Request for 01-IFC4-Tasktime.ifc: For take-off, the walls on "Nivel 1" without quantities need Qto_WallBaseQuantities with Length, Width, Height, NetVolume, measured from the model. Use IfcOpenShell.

First a look at what the model holds.

```python
import ifcopenshell
import ifcopenshell.util.element
import ifcopenshell.util.unit

model = ifcopenshell.open("01-IFC4-Tasktime.ifc")
print(model.schema)
for unit_type in ("LENGTHUNIT", "AREAUNIT", "VOLUMEUNIT"):
    print(unit_type, ifcopenshell.util.unit.calculate_unit_scale(model, unit_type))
storey = next(s for s in model.by_type("IfcBuildingStorey") if s.Name == "Nivel 1")
walls = [e for e in ifcopenshell.util.element.get_decomposition(storey) if e.is_a("IfcWall")]
for e in sorted(walls, key=lambda e: e.id()):
    print(e.id(), e.is_a(), e.Name, list(ifcopenshell.util.element.get_psets(e, qtos_only=True)), sep=" | ")
```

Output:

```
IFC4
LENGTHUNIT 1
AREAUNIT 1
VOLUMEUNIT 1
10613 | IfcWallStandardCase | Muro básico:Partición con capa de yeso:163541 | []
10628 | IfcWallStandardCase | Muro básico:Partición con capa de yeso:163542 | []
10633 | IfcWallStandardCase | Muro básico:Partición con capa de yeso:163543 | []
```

```python
import ifcopenshell
import ifcopenshell.api.pset
import ifcopenshell.geom
import ifcopenshell.util.element
import ifcopenshell.util.shape
import ifcopenshell.util.unit

model = ifcopenshell.open("01-IFC4-Tasktime.ifc")
unit_scale = ifcopenshell.util.unit.calculate_unit_scale(model)
volume_scale = ifcopenshell.util.unit.calculate_unit_scale(model, "VOLUMEUNIT")
settings = ifcopenshell.geom.settings()

storey = next(s for s in model.by_type("IfcBuildingStorey") if s.Name == "Nivel 1")
walls = [e for e in ifcopenshell.util.element.get_decomposition(storey) if e.is_a("IfcWall")]

for e in sorted(walls, key=lambda e: e.id()):
    if ifcopenshell.util.element.get_psets(e, qtos_only=True, should_inherit=False):
        continue
    # Geometry comes back in metres, in the element's own axes.
    shape = ifcopenshell.geom.create_shape(settings, e)
    values = {
        "Length": ifcopenshell.util.shape.get_x(shape.geometry) / unit_scale,
        "Width": ifcopenshell.util.shape.get_y(shape.geometry) / unit_scale,
        "Height": ifcopenshell.util.shape.get_z(shape.geometry) / unit_scale,
        "NetVolume": ifcopenshell.util.shape.get_volume(shape.geometry) / volume_scale,
    }
    qto = ifcopenshell.api.pset.add_qto(model, product=e, name="Qto_WallBaseQuantities")
    ifcopenshell.api.pset.edit_qto(model, qto=qto, properties=values)
    print(e.id(), {k: round(v, 3) for k, v in values.items()})

model.write("01-IFC4-Tasktime-out.ifc")
```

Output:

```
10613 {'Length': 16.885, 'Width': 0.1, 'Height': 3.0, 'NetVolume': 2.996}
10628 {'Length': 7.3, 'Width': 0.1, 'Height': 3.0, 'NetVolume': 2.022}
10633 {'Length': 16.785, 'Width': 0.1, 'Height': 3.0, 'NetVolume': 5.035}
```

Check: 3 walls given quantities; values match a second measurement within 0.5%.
